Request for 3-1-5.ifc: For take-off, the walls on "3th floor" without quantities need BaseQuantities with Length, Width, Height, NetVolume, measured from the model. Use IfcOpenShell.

First a look at what the model holds.

```python
import ifcopenshell
import ifcopenshell.util.element
import ifcopenshell.util.unit

model = ifcopenshell.open("3-1-5.ifc")
print(model.schema)
for unit_type in ("LENGTHUNIT", "AREAUNIT", "VOLUMEUNIT"):
    print(unit_type, ifcopenshell.util.unit.calculate_unit_scale(model, unit_type))
storey = next(s for s in model.by_type("IfcBuildingStorey") if s.Name == "3th floor")
walls = [e for e in ifcopenshell.util.element.get_decomposition(storey) if e.is_a("IfcWall")]
for e in sorted(walls, key=lambda e: e.id()):
    print(e.id(), e.is_a(), e.Name, list(ifcopenshell.util.element.get_psets(e, qtos_only=True)), sep=" | ")
```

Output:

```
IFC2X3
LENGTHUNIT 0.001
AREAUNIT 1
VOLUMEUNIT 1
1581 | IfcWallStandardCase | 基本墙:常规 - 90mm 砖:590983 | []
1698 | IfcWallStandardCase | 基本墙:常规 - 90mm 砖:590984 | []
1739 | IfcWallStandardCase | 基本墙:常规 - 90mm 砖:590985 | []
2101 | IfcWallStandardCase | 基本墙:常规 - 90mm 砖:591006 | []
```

```python
import ifcopenshell
import ifcopenshell.api.pset
import ifcopenshell.geom
import ifcopenshell.util.element
import ifcopenshell.util.shape
import ifcopenshell.util.unit

model = ifcopenshell.open("3-1-5.ifc")
unit_scale = ifcopenshell.util.unit.calculate_unit_scale(model)
volume_scale = ifcopenshell.util.unit.calculate_unit_scale(model, "VOLUMEUNIT")
settings = ifcopenshell.geom.settings()

storey = next(s for s in model.by_type("IfcBuildingStorey") if s.Name == "3th floor")
walls = [e for e in ifcopenshell.util.element.get_decomposition(storey) if e.is_a("IfcWall")]

for e in sorted(walls, key=lambda e: e.id()):
    if ifcopenshell.util.element.get_psets(e, qtos_only=True, should_inherit=False):
        continue
    # Geometry comes back in metres, in the element's own axes.
    shape = ifcopenshell.geom.create_shape(settings, e)
    values = {
        "Length": ifcopenshell.util.shape.get_x(shape.geometry) / unit_scale,
        "Width": ifcopenshell.util.shape.get_y(shape.geometry) / unit_scale,
        "Height": ifcopenshell.util.shape.get_z(shape.geometry) / unit_scale,
        "NetVolume": ifcopenshell.util.shape.get_volume(shape.geometry) / volume_scale,
    }
    qto = ifcopenshell.api.pset.add_qto(model, product=e, name="BaseQuantities")
    ifcopenshell.api.pset.edit_qto(model, qto=qto, properties=values)
    print(e.id(), {k: round(v, 3) for k, v in values.items()})

model.write("3-1-5-out.ifc")
```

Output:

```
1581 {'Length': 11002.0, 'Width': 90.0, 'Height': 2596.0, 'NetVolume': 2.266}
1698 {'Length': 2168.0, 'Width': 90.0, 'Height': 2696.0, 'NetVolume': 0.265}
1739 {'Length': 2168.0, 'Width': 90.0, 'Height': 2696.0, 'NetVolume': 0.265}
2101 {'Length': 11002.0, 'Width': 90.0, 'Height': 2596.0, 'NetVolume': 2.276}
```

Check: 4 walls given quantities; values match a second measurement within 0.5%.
